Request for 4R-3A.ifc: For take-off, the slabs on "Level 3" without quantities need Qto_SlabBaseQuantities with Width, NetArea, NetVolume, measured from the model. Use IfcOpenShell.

First a look at what the model holds.

```python
import ifcopenshell
import ifcopenshell.util.element
import ifcopenshell.util.unit

model = ifcopenshell.open("4R-3A.ifc")
print(model.schema)
for unit_type in ("LENGTHUNIT", "AREAUNIT", "VOLUMEUNIT"):
    print(unit_type, ifcopenshell.util.unit.calculate_unit_scale(model, unit_type))
storey = next(s for s in model.by_type("IfcBuildingStorey") if s.Name == "Level 3")
slabs = [e for e in ifcopenshell.util.element.get_decomposition(storey) if e.is_a("IfcSlab")]
for e in sorted(slabs, key=lambda e: e.id()):
    print(e.id(), e.is_a(), e.Name, list(ifcopenshell.util.element.get_psets(e, qtos_only=True)), sep=" | ")
```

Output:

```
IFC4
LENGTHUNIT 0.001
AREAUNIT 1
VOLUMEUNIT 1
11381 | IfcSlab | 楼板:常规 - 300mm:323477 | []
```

```python
import ifcopenshell
import ifcopenshell.api.pset
import ifcopenshell.geom
import ifcopenshell.util.element
import ifcopenshell.util.shape
import ifcopenshell.util.unit

model = ifcopenshell.open("4R-3A.ifc")
unit_scale = ifcopenshell.util.unit.calculate_unit_scale(model)
area_scale = ifcopenshell.util.unit.calculate_unit_scale(model, "AREAUNIT")
volume_scale = ifcopenshell.util.unit.calculate_unit_scale(model, "VOLUMEUNIT")
settings = ifcopenshell.geom.settings()

storey = next(s for s in model.by_type("IfcBuildingStorey") if s.Name == "Level 3")
slabs = [e for e in ifcopenshell.util.element.get_decomposition(storey) if e.is_a("IfcSlab")]

for e in sorted(slabs, key=lambda e: e.id()):
    if ifcopenshell.util.element.get_psets(e, qtos_only=True, should_inherit=False):
        continue
    # Geometry comes back in metres, in the element's own axes.
    shape = ifcopenshell.geom.create_shape(settings, e)
    values = {
        "Width": ifcopenshell.util.shape.get_z(shape.geometry) / unit_scale,
        "NetArea": ifcopenshell.util.shape.get_footprint_area(shape.geometry) / area_scale,
        "NetVolume": ifcopenshell.util.shape.get_volume(shape.geometry) / volume_scale,
    }
    qto = ifcopenshell.api.pset.add_qto(model, product=e, name="Qto_SlabBaseQuantities")
    ifcopenshell.api.pset.edit_qto(model, qto=qto, properties=values)
    print(e.id(), {k: round(v, 3) for k, v in values.items()})

model.write("4R-3A_v2.ifc")
```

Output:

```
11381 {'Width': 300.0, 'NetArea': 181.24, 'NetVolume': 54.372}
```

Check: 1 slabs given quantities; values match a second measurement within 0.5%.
